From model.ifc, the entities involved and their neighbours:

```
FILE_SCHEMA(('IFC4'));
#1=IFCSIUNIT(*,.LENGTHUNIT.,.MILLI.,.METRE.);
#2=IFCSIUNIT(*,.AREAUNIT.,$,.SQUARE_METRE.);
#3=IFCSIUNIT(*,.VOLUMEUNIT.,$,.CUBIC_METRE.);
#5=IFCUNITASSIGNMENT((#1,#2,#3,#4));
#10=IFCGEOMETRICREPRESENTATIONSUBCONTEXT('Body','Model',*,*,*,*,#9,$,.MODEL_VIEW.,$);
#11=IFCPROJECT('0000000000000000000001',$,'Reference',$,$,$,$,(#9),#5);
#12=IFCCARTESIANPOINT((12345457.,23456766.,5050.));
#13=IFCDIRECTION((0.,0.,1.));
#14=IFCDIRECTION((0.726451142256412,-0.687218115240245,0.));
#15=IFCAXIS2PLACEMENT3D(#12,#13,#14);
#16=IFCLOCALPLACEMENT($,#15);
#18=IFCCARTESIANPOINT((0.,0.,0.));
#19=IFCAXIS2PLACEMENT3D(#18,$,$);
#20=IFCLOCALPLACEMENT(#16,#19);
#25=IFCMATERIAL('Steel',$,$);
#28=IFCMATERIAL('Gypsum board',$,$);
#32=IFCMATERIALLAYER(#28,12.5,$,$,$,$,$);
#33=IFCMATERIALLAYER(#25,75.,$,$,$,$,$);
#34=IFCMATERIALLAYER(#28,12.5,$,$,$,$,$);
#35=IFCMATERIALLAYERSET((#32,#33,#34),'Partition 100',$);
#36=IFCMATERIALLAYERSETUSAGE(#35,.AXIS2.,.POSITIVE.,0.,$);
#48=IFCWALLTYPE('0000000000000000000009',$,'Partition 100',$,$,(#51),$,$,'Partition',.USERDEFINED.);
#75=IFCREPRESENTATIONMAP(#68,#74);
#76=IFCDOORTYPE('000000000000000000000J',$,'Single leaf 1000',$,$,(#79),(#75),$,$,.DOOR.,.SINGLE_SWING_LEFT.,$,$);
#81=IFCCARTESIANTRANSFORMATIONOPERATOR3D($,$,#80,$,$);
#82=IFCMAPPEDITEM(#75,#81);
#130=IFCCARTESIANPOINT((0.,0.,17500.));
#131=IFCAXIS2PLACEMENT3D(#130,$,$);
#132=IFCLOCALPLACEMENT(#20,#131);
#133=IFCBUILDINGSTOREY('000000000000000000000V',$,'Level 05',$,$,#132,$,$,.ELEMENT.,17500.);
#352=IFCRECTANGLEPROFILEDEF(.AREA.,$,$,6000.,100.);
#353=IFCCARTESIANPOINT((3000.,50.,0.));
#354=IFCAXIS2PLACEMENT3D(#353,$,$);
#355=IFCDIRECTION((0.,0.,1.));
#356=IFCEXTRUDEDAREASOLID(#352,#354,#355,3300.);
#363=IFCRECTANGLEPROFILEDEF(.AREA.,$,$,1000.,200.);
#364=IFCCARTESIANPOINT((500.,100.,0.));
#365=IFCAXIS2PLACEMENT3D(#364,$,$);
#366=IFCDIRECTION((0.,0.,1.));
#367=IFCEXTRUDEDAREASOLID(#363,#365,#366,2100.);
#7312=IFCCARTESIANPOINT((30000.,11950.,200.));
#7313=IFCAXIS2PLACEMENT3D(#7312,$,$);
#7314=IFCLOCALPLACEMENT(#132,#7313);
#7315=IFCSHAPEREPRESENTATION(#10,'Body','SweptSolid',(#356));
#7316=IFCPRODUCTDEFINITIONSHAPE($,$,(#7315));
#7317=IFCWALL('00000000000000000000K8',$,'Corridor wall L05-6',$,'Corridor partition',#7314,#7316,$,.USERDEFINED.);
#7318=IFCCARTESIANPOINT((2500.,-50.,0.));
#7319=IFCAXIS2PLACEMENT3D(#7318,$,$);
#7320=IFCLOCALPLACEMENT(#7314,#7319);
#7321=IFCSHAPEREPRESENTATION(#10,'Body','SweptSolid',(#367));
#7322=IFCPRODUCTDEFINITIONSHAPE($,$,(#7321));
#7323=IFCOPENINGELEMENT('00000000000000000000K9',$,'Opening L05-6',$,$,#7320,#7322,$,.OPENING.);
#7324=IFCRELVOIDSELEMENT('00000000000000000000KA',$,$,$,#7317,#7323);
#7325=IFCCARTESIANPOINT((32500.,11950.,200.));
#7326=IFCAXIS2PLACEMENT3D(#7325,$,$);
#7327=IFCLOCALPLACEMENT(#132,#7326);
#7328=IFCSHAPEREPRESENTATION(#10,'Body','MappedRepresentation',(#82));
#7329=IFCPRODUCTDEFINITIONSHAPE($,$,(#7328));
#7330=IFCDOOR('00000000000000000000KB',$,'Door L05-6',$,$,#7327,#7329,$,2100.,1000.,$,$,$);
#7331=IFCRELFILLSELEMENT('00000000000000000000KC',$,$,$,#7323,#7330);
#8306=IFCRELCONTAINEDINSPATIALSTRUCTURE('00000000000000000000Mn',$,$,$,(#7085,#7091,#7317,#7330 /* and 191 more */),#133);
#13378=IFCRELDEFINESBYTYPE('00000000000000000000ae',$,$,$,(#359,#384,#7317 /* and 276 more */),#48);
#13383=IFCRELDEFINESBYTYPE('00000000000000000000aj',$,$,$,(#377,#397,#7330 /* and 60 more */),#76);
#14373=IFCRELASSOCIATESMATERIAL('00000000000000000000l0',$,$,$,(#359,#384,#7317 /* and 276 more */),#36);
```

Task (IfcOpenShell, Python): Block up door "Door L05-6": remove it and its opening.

```python
import ifcopenshell
import ifcopenshell.api.feature
import ifcopenshell.api.root
import ifcopenshell.geom
import ifcopenshell.util.shape

model = ifcopenshell.open("model.ifc")
settings = ifcopenshell.geom.settings()


def volume(element):
    """Net volume in cubic metres, openings subtracted."""
    shape = ifcopenshell.geom.create_shape(settings, element)
    return ifcopenshell.util.shape.get_volume(shape.geometry)


door = model.by_id(7330)
opening = door.FillsVoids[0].RelatingOpeningElement
wall = opening.VoidsElements[0].RelatingBuildingElement
before = volume(wall)

ifcopenshell.api.root.remove_product(model, product=door)
ifcopenshell.api.feature.remove_feature(model, feature=opening)

after = volume(wall)

print(f"wall volume {before:.3f} -> {after:.3f} m3")

model.write("model_updated.ifc")
```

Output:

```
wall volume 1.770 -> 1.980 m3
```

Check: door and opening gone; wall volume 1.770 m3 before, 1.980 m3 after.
